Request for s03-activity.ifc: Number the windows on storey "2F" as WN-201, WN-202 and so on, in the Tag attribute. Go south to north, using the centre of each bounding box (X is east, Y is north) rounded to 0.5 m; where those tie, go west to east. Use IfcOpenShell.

First a look at what the model holds.

```python
import ifcopenshell
import ifcopenshell.util.element
import ifcopenshell.util.placement

model = ifcopenshell.open("s03-activity.ifc")
print(model.schema)
storey = next(s for s in model.by_type("IfcBuildingStorey") if s.Name == "2F")
windows = [e for e in ifcopenshell.util.element.get_decomposition(storey) if e.is_a("IfcWindow")]
for e in sorted(windows, key=lambda e: e.id()):
    origin = ifcopenshell.util.placement.get_local_placement(e.ObjectPlacement)[:3, 3]
    print(e.id(), e.Tag, e.Name, origin.round(2) + 0.0, sep=" | ")
```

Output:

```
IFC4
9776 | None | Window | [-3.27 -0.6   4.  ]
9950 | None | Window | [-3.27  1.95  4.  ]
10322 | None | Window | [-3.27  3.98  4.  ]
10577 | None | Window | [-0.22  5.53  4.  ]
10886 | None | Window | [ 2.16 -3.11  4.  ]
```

```python
import ifcopenshell
import ifcopenshell.geom
import ifcopenshell.util.element
import ifcopenshell.util.shape

model = ifcopenshell.open("s03-activity.ifc")
settings = ifcopenshell.geom.settings()
settings.set("use-world-coords", True)


def centre(element):
    shape = ifcopenshell.geom.create_shape(settings, element)
    return ifcopenshell.util.shape.get_bbox_centroid(shape.geometry)


storey = next(s for s in model.by_type("IfcBuildingStorey") if s.Name == "2F")
windows = [e for e in ifcopenshell.util.element.get_decomposition(storey) if e.is_a("IfcWindow")]

# Insertion points can sit at a corner or the storey origin, so sort by the geometry (in metres).
centres = {e: centre(e) for e in windows}
windows.sort(key=lambda e: (round(centres[e][1] / 0.5), centres[e][0]))

for i, e in enumerate(windows, start=1):
    number = f"WN-2{i:02d}"
    e.Tag = number
    print(e.id(), number)

model.write("s03-activity_edited.ifc")
```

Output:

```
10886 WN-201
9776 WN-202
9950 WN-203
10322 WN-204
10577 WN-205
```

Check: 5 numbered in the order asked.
